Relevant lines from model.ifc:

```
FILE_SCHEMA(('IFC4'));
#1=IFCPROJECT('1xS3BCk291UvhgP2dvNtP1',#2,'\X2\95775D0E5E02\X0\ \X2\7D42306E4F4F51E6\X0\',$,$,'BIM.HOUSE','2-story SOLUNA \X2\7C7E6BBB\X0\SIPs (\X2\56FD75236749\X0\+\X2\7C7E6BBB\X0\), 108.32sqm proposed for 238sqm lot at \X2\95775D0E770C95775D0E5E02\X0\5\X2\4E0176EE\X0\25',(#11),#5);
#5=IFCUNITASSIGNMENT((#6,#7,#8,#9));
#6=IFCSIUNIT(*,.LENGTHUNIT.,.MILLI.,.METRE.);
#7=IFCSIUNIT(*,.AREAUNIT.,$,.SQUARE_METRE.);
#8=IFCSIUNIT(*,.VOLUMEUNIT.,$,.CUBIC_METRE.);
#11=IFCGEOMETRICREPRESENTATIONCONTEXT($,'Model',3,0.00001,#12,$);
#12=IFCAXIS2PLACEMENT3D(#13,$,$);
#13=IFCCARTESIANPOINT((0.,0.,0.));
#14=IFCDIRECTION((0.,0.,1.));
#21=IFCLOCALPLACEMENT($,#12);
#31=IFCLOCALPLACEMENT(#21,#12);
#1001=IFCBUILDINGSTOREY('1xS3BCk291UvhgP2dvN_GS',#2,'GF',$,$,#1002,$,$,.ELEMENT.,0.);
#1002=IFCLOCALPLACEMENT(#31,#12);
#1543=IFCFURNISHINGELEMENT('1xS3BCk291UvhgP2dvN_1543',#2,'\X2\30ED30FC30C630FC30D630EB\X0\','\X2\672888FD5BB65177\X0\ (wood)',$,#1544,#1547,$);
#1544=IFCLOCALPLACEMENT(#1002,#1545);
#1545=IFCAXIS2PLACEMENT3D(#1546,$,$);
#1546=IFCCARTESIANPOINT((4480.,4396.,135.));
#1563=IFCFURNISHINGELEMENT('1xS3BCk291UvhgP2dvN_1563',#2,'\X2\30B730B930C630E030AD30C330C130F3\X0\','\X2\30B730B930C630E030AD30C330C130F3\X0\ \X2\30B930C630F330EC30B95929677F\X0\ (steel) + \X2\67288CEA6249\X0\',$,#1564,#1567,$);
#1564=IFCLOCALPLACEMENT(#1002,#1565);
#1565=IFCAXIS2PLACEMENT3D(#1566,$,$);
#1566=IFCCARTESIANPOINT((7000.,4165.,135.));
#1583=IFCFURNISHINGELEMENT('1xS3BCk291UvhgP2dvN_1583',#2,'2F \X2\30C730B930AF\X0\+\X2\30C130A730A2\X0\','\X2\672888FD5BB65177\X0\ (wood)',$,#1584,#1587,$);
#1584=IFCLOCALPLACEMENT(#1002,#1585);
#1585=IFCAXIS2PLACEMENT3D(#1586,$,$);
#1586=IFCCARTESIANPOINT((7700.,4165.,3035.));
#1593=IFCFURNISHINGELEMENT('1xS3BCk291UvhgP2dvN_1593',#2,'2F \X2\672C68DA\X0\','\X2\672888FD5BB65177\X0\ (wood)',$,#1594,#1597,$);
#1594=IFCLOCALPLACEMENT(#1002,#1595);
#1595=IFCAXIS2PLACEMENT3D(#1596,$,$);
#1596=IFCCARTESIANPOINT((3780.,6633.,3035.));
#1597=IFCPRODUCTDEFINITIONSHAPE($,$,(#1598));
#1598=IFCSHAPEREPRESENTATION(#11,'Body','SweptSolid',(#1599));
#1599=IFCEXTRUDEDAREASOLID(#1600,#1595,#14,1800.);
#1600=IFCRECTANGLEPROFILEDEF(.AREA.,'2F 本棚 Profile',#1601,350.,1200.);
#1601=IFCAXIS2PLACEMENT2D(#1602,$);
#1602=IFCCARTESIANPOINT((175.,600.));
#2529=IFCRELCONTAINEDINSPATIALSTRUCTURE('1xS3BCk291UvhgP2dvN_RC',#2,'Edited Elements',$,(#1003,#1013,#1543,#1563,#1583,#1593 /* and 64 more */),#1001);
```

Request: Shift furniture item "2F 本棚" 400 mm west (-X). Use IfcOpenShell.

```python
import ifcopenshell
import ifcopenshell.api.geometry
import ifcopenshell.util.placement
import ifcopenshell.util.unit

model = ifcopenshell.open("model.ifc")
unit_scale = ifcopenshell.util.unit.calculate_unit_scale(model)

item = model.by_id(1593)
matrix = ifcopenshell.util.placement.get_local_placement(item.ObjectPlacement)
matrix[0, 3] -= 0.4 / unit_scale
ifcopenshell.api.geometry.edit_object_placement(model, product=item, matrix=matrix, is_si=False)

print(ifcopenshell.util.placement.get_local_placement(item.ObjectPlacement).round(3) + 0.0)

model.write("model_updated.ifc")
```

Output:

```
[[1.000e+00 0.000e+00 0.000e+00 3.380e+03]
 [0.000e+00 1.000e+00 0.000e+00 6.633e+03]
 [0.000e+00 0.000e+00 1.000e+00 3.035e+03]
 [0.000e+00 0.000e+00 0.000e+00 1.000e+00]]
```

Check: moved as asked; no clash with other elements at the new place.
